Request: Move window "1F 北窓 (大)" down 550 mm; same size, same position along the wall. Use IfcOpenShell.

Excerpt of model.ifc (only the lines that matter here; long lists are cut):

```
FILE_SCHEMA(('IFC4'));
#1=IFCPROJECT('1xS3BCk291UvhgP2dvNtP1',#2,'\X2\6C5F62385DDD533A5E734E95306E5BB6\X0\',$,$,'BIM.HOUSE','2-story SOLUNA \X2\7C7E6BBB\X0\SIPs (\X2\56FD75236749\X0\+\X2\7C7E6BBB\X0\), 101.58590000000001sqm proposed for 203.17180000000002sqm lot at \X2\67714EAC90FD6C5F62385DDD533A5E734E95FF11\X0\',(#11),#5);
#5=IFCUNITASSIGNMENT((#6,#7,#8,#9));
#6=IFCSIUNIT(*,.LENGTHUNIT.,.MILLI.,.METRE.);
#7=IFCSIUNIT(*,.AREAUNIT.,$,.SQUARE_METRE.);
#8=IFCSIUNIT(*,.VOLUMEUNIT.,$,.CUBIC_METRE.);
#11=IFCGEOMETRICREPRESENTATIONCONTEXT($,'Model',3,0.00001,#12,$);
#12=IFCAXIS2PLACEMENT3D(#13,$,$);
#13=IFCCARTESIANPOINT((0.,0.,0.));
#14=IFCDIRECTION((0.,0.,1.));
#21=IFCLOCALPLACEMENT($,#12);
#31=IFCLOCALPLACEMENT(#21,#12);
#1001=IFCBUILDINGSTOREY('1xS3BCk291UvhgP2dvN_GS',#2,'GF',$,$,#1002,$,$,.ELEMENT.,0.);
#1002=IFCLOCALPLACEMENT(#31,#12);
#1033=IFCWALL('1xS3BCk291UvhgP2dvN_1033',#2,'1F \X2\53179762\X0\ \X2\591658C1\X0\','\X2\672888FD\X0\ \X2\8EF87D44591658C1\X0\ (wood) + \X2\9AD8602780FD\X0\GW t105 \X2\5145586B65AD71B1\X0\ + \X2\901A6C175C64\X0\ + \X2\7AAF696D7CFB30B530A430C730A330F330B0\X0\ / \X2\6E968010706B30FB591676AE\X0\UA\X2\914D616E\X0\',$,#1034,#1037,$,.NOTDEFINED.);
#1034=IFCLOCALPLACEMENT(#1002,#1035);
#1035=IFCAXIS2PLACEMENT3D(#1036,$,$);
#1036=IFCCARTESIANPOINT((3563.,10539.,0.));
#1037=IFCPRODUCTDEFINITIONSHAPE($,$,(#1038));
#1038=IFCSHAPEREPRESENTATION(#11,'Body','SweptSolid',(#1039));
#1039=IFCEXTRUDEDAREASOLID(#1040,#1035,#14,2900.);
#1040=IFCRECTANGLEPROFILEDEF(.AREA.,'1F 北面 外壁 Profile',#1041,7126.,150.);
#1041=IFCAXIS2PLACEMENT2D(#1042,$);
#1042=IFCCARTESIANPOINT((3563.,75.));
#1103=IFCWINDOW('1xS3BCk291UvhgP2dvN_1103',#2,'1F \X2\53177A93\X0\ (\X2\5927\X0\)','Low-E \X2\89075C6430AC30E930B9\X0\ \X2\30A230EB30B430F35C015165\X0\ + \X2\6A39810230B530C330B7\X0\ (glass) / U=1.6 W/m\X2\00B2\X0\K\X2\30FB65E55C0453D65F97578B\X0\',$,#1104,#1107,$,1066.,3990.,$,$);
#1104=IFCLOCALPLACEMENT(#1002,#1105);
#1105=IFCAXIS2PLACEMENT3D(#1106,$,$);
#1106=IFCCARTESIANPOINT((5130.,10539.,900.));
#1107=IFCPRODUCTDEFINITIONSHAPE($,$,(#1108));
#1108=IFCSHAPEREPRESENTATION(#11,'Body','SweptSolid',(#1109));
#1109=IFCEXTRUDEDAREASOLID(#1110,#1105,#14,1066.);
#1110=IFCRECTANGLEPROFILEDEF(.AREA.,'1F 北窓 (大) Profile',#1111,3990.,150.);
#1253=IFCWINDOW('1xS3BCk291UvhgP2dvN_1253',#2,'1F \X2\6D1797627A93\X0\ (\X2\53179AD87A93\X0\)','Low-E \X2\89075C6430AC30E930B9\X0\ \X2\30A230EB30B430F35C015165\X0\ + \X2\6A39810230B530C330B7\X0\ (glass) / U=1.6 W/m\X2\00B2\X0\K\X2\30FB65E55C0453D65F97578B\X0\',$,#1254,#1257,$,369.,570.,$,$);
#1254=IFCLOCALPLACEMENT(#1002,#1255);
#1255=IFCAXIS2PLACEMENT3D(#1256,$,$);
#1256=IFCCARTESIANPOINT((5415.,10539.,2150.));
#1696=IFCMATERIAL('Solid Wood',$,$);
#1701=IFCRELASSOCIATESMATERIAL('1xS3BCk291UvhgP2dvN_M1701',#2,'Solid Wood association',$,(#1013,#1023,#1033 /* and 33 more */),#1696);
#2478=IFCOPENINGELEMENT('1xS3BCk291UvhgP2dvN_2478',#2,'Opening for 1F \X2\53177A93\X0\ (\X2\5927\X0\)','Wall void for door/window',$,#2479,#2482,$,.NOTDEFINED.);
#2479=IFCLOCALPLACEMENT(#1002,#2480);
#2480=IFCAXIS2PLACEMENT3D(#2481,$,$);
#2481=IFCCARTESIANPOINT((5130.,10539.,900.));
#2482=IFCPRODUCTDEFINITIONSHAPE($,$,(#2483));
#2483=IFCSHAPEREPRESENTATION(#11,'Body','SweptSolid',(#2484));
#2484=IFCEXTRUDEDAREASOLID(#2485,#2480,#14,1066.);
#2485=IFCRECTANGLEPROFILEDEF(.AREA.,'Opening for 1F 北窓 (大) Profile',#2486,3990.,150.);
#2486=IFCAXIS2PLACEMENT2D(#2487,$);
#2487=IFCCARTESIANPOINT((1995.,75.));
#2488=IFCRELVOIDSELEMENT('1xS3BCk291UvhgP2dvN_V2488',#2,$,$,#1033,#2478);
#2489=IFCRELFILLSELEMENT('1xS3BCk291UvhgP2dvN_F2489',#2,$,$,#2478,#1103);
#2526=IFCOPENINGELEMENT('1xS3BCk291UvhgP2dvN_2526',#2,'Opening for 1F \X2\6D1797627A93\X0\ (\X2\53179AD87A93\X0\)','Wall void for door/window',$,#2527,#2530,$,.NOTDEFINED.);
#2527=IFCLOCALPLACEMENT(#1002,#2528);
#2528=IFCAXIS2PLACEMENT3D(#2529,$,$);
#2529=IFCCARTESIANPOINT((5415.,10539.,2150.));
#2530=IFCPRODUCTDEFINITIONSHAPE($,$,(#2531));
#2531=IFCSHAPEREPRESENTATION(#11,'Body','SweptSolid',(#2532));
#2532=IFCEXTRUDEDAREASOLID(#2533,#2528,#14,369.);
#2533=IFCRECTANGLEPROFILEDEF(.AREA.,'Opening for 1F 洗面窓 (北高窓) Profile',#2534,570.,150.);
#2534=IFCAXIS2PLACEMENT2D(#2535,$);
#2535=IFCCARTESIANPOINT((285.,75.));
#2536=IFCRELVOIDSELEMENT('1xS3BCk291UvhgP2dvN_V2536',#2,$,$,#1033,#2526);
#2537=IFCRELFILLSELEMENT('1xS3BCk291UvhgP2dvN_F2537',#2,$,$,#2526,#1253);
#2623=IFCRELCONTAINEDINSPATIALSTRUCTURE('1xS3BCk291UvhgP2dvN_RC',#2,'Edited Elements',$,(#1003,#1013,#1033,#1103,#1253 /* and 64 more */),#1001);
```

```python
import numpy as np
import ifcopenshell
import ifcopenshell.api.geometry
import ifcopenshell.util.placement
import ifcopenshell.util.unit

model = ifcopenshell.open("model.ifc")
unit_scale = ifcopenshell.util.unit.calculate_unit_scale(model)

window = model.by_guid("1xS3BCk291UvhgP2dvN_1103")
opening = window.FillsVoids[0].RelatingOpeningElement
dz = -550.0

shift = np.array([0.0, 0.0, dz])
# The window is not placed relative to its opening, so move both.
for product in (opening, window):
    matrix = ifcopenshell.util.placement.get_local_placement(product.ObjectPlacement)
    matrix[:3, 3] += shift
    ifcopenshell.api.geometry.edit_object_placement(model, product=product, matrix=matrix, is_si=False)

print(f"moved by {dz * unit_scale:+.3f} m")

model.write("model_edited.ifc")
```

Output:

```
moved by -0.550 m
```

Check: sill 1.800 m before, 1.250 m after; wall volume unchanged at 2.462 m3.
